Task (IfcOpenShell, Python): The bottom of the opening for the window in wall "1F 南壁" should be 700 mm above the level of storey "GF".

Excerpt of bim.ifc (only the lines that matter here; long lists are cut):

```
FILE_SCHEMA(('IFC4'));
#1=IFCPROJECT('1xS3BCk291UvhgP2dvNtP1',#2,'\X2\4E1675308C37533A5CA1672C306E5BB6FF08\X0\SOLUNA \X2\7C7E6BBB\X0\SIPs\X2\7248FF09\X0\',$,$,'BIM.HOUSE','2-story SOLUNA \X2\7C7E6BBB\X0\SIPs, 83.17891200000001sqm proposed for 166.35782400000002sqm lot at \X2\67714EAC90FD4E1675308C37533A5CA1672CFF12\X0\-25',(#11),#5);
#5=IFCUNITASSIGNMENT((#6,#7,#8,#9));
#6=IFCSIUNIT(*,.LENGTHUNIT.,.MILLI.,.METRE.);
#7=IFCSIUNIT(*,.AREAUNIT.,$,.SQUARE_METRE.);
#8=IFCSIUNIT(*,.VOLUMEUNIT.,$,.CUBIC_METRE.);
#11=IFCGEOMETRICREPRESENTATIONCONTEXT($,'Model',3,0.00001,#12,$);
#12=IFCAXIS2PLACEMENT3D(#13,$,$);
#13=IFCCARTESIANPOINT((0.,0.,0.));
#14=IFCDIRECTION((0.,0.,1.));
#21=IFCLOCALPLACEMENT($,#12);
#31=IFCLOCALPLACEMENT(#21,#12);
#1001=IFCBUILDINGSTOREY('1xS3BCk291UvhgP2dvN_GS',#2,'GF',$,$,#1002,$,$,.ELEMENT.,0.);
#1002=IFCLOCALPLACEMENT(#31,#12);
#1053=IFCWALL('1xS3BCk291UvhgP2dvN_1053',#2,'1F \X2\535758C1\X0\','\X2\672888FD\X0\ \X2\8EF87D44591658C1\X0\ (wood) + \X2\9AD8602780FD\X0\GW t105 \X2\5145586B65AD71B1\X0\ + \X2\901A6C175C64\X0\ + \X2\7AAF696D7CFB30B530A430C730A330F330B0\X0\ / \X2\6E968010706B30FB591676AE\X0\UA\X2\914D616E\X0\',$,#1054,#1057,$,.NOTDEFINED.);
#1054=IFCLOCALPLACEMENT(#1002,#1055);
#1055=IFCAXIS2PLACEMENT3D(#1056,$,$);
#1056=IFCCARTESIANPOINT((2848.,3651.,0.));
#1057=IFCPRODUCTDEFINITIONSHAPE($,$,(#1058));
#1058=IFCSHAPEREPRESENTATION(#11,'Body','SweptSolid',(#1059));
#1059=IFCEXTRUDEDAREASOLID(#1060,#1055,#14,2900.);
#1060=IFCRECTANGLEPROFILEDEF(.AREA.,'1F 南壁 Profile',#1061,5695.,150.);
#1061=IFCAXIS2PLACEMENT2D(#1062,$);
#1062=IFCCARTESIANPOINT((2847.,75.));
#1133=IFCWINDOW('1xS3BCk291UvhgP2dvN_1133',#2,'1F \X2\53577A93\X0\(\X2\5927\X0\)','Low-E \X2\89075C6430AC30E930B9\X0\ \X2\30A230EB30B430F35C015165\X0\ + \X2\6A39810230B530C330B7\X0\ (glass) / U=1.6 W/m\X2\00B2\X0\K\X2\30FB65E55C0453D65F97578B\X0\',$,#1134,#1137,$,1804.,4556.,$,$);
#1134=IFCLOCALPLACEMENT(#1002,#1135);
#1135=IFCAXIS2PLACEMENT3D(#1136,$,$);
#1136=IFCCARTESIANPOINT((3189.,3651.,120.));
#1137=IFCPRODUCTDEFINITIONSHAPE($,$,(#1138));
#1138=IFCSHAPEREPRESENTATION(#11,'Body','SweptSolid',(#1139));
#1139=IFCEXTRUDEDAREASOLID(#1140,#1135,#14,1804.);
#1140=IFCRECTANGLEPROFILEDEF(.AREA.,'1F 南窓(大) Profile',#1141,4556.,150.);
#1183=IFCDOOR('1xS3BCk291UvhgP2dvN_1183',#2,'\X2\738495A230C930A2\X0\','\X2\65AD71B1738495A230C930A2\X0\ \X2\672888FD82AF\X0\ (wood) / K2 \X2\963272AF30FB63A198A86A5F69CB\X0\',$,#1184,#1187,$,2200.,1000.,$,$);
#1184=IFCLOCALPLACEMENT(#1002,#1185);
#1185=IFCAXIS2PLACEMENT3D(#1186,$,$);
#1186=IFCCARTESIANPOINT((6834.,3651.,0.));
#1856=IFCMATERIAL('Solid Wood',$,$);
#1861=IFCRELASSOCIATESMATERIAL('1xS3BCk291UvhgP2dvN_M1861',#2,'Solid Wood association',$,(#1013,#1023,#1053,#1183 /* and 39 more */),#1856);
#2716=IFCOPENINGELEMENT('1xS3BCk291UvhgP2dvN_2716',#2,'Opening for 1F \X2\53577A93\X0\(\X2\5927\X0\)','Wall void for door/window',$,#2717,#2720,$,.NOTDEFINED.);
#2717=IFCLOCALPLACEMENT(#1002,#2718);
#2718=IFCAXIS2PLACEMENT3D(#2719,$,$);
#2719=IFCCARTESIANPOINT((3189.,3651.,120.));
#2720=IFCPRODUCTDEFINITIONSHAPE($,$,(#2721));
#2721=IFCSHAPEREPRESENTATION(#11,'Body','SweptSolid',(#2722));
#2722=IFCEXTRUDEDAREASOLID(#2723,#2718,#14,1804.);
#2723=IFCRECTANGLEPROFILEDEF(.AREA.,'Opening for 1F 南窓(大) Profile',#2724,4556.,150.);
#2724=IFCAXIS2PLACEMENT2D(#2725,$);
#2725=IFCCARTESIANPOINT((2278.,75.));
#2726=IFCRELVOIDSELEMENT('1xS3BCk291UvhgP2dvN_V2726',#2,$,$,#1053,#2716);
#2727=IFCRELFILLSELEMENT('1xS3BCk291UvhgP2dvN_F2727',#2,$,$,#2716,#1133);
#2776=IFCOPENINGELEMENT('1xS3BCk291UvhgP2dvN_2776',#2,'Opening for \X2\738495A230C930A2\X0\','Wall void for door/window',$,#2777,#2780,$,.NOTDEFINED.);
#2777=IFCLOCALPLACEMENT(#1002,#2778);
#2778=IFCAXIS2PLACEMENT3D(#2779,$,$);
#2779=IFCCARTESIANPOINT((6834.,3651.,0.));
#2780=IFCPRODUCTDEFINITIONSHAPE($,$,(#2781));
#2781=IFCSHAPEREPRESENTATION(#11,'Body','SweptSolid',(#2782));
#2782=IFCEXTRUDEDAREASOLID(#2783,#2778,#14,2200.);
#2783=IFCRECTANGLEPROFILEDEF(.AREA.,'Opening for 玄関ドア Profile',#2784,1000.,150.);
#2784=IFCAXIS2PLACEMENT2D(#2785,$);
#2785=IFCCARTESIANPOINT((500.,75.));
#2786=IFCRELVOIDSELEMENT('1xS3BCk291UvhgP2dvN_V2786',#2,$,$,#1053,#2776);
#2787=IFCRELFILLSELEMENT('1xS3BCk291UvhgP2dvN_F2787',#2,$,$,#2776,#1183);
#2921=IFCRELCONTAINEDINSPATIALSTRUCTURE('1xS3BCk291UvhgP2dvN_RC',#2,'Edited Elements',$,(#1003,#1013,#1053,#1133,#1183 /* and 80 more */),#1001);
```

```python
import numpy as np
import ifcopenshell
import ifcopenshell.api.geometry
import ifcopenshell.geom
import ifcopenshell.util.element
import ifcopenshell.util.placement
import ifcopenshell.util.shape
import ifcopenshell.util.unit

model = ifcopenshell.open("bim.ifc")
unit_scale = ifcopenshell.util.unit.calculate_unit_scale(model)

window = model.by_id(1133)
opening = window.FillsVoids[0].RelatingOpeningElement
storey = ifcopenshell.util.element.get_container(window, ifc_class="IfcBuildingStorey")
level = ifcopenshell.util.placement.get_local_placement(storey.ObjectPlacement)[2, 3]

# The opening's origin need not be at the sill, so measure its lowest point.
shape = ifcopenshell.geom.create_shape(ifcopenshell.geom.settings(), opening)
bottom = ifcopenshell.util.shape.get_shape_bottom_elevation(shape, shape.geometry) / unit_scale
dz = level + 0.7 / unit_scale - bottom

shift = np.array([0.0, 0.0, dz])
# The window is not placed relative to its opening, so move both.
for product in (opening, window):
    matrix = ifcopenshell.util.placement.get_local_placement(product.ObjectPlacement)
    matrix[:3, 3] += shift
    ifcopenshell.api.geometry.edit_object_placement(model, product=product, matrix=matrix, is_si=False)

print(f"moved by {dz * unit_scale:+.3f} m")

model.write("bim_rev.ifc")
```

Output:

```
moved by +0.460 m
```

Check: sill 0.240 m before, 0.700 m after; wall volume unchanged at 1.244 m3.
